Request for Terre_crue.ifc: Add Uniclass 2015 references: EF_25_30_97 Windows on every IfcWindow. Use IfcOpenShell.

First a look at what the model holds.

```python
import ifcopenshell

model = ifcopenshell.open("Terre_crue.ifc")
print(model.schema)
print("classifications:", [c.Name for c in model.by_type("IfcClassification")])
for ifc_class in ("IfcDoor", "IfcRoof", "IfcStair", "IfcWall", "IfcWindow"):
    print(ifc_class, len(model.by_type(ifc_class)))
```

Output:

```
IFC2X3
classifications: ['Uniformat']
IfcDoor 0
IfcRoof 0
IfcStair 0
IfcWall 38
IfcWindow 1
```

```python
import ifcopenshell
import ifcopenshell.api.classification

model = ifcopenshell.open("Terre_crue.ifc")

# IFC2X3 requires Source and Edition and has no link from the project to the system.
system = model.create_entity("IfcClassification", Source="NBS", Edition="2015", Name="Uniclass 2015")

codes = {
    "IfcWindow": ("EF_25_30_97", "Windows"),
}
for ifc_class, (code, name) in codes.items():
    products = model.by_type(ifc_class)
    ifcopenshell.api.classification.add_reference(
        model, products=products, classification=system, identification=code, name=name
    )
    print(code, len(products))

model.write("Terre_crue_rev.ifc")
```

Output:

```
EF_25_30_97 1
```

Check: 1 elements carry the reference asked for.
